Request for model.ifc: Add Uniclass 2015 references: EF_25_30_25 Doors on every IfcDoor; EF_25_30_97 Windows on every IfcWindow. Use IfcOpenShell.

First a look at what the model holds.

```python
import ifcopenshell

model = ifcopenshell.open("model.ifc")
print(model.schema)
print("classifications:", [c.Name for c in model.by_type("IfcClassification")])
for ifc_class in ("IfcDoor", "IfcRoof", "IfcStair", "IfcWall", "IfcWindow"):
    print(ifc_class, len(model.by_type(ifc_class)))
```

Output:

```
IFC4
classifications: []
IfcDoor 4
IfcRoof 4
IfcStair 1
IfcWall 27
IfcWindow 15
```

```python
import ifcopenshell
import ifcopenshell.api.classification

model = ifcopenshell.open("model.ifc")

system = ifcopenshell.api.classification.add_classification(model, classification="Uniclass 2015")

codes = {
    "IfcDoor": ("EF_25_30_25", "Doors"),
    "IfcWindow": ("EF_25_30_97", "Windows"),
}
for ifc_class, (code, name) in codes.items():
    products = model.by_type(ifc_class)
    ifcopenshell.api.classification.add_reference(
        model, products=products, classification=system, identification=code, name=name
    )
    print(code, len(products))

model.write("model_updated.ifc")
```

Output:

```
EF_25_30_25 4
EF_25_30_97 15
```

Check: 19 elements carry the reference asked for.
